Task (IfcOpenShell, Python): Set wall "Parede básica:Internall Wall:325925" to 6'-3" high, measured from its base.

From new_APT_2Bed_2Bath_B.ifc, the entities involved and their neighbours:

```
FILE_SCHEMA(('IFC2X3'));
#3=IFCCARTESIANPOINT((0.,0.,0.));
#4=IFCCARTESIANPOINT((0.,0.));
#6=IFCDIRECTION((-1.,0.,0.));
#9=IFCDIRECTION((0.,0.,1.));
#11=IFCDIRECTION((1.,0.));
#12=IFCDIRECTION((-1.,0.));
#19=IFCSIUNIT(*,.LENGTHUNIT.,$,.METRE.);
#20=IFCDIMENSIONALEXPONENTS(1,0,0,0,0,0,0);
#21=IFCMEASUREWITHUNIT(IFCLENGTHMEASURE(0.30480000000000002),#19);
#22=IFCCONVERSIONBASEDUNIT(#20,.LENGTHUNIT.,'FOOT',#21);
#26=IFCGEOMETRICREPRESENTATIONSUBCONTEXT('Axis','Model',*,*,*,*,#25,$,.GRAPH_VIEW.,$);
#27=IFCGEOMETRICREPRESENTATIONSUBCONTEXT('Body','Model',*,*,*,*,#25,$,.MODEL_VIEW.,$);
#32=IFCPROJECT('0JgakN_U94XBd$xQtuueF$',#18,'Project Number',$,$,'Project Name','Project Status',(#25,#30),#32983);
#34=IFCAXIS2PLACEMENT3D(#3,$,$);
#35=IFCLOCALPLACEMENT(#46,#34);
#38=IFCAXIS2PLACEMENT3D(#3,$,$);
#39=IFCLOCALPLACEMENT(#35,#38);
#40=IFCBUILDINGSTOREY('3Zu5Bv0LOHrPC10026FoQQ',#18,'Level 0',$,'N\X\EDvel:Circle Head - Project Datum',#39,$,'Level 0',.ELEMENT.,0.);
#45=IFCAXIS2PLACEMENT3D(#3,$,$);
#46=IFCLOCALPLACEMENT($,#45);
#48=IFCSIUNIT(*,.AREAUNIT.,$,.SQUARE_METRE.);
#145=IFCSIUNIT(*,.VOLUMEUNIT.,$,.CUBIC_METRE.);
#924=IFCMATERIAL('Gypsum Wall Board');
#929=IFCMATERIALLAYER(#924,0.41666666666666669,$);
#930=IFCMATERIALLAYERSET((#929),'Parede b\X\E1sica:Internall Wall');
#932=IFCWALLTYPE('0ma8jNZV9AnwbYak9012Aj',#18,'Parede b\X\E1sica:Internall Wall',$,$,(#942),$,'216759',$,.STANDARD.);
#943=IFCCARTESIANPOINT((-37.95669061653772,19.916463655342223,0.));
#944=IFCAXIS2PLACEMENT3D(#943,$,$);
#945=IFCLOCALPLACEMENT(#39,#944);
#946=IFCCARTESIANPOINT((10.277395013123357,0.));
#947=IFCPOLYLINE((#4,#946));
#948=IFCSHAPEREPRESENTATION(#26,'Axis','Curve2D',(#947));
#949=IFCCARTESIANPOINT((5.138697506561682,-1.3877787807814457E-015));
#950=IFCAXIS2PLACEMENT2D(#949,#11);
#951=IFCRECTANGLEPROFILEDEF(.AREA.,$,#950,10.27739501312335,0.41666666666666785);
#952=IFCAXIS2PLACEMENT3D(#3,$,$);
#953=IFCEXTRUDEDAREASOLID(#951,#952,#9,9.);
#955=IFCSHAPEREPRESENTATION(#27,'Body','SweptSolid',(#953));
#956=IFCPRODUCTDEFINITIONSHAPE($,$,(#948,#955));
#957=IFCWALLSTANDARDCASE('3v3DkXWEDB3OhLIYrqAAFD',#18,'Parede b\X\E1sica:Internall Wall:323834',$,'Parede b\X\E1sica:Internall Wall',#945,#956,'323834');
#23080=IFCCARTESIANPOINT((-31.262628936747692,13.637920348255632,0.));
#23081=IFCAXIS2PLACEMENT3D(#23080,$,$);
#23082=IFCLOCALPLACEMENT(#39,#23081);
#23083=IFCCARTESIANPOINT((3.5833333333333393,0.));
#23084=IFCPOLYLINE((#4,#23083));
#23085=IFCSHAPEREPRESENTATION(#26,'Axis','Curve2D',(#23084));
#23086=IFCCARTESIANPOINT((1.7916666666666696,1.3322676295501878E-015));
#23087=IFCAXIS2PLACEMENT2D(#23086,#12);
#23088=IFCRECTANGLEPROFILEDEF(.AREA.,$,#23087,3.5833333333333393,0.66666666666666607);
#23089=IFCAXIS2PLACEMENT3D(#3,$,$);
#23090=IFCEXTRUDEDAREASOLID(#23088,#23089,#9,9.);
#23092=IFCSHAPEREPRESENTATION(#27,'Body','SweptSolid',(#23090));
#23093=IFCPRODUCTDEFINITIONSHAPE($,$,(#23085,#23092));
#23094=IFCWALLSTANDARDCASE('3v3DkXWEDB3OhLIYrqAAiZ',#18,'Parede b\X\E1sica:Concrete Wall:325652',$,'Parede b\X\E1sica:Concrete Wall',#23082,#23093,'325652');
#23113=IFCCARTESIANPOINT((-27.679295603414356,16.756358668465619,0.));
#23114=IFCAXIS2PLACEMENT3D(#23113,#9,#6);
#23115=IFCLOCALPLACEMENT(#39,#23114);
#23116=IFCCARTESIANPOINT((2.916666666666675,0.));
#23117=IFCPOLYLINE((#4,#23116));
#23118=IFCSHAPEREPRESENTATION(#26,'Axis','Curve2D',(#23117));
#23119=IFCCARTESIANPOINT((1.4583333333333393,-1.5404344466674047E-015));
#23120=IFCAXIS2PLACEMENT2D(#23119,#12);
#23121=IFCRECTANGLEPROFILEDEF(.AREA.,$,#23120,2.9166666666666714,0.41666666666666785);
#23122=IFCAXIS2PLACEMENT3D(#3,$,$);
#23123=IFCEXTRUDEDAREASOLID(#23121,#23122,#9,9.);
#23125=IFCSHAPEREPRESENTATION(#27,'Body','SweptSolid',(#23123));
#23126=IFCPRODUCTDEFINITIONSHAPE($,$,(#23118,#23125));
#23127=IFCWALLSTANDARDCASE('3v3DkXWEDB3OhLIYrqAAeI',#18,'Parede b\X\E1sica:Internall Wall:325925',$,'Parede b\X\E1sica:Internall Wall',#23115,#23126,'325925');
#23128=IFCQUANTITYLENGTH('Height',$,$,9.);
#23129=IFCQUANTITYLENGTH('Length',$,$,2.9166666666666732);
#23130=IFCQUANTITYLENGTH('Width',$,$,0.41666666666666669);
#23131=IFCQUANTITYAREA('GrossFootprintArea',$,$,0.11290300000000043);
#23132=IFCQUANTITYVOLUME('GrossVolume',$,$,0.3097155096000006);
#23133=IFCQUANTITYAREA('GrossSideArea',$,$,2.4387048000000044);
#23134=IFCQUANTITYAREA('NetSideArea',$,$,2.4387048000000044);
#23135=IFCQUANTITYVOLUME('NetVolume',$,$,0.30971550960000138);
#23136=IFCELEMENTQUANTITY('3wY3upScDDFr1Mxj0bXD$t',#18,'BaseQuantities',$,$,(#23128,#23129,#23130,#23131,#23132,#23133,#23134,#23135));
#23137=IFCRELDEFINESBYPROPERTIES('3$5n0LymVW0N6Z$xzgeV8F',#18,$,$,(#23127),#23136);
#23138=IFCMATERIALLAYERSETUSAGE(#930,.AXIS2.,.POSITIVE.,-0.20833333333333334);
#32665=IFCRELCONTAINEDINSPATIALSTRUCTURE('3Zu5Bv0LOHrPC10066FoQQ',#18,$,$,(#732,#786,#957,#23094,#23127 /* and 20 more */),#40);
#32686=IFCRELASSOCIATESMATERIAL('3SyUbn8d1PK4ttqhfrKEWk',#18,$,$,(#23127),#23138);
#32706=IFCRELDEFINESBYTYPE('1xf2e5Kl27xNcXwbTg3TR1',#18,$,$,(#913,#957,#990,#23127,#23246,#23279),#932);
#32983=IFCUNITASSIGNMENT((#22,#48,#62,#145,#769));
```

```python
import ifcopenshell
import ifcopenshell.api.pset
import ifcopenshell.geom
import ifcopenshell.util.element
import ifcopenshell.util.representation
import ifcopenshell.util.shape
import ifcopenshell.util.unit

model = ifcopenshell.open("new_APT_2Bed_2Bath_B.ifc")
unit_scale = ifcopenshell.util.unit.calculate_unit_scale(model)
area_scale = ifcopenshell.util.unit.calculate_unit_scale(model, "AREAUNIT")
volume_scale = ifcopenshell.util.unit.calculate_unit_scale(model, "VOLUMEUNIT")
settings = ifcopenshell.geom.settings()


def volume(element):
    """Net volume in cubic metres, openings subtracted."""
    shape = ifcopenshell.geom.create_shape(settings, element)
    return ifcopenshell.util.shape.get_volume(shape.geometry)


wall = model.by_guid("3v3DkXWEDB3OhLIYrqAAeI")
before = volume(wall)

body = ifcopenshell.util.representation.get_representation(wall, "Model", "Body")
solid = body.Items[0]
old_height = solid.Depth
solid.Depth = 75 * 0.0254 / unit_scale
after = volume(wall)
thickness = 0.127  # wall thickness in metres

# Update the stored height, areas and volumes.
qto = model.by_id(ifcopenshell.util.element.get_pset(wall, "BaseQuantities", should_inherit=False)["id"])
ifcopenshell.api.pset.edit_qto(model, qto=qto, properties={
    "Height": solid.Depth,
    "GrossVolume": ifcopenshell.util.element.get_pset(wall, "BaseQuantities", "GrossVolume") * solid.Depth / old_height,
    "GrossSideArea": ifcopenshell.util.element.get_pset(wall, "BaseQuantities", "GrossSideArea") * solid.Depth / old_height,
    "NetSideArea": after / thickness / area_scale,
    "NetVolume": after / volume_scale,
})

print(f"height {old_height:g} -> {solid.Depth:g}, volume {before:.3f} -> {after:.3f} m3")

model.write("new_APT_2Bed_2Bath_B_v2.ifc")
```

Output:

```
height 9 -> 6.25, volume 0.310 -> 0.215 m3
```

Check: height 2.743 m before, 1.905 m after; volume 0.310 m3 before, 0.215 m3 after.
